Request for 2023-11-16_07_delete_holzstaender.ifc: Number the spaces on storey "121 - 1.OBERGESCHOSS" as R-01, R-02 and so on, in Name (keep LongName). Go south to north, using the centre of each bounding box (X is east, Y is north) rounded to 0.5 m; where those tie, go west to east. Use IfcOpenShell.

First a look at what the model holds.

```python
import ifcopenshell
import ifcopenshell.util.element
import ifcopenshell.util.placement

model = ifcopenshell.open("2023-11-16_07_delete_holzstaender.ifc")
print(model.schema)
storey = next(s for s in model.by_type("IfcBuildingStorey") if s.Name == "121 - 1.OBERGESCHOSS")
spaces = [e for e in ifcopenshell.util.element.get_decomposition(storey) if e.is_a("IfcSpace")]
for e in sorted(spaces, key=lambda e: e.id()):
    origin = ifcopenshell.util.placement.get_local_placement(e.ObjectPlacement)[:3, 3]
    print(e.id(), e.Name, e.LongName, origin.round(2) + 0.0, sep=" | ")
```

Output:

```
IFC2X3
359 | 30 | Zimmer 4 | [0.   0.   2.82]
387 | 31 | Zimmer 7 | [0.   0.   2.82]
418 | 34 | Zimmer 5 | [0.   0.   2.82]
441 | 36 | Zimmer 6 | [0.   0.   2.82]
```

```python
import ifcopenshell
import ifcopenshell.geom
import ifcopenshell.util.element
import ifcopenshell.util.shape

model = ifcopenshell.open("2023-11-16_07_delete_holzstaender.ifc")
settings = ifcopenshell.geom.settings()
settings.set("use-world-coords", True)


def centre(element):
    shape = ifcopenshell.geom.create_shape(settings, element)
    return ifcopenshell.util.shape.get_bbox_centroid(shape.geometry)


storey = next(s for s in model.by_type("IfcBuildingStorey") if s.Name == "121 - 1.OBERGESCHOSS")
spaces = [e for e in ifcopenshell.util.element.get_decomposition(storey) if e.is_a("IfcSpace")]

# Insertion points can sit at a corner or the storey origin, so sort by the geometry (in metres).
centres = {e: centre(e) for e in spaces}
spaces.sort(key=lambda e: (round(centres[e][1] / 0.5), centres[e][0]))

for i, e in enumerate(spaces, start=1):
    number = f"R-{i:02d}"
    e.Name = number
    print(e.id(), number)

model.write("2023-11-16_07_delete_holzstaender-out.ifc")
```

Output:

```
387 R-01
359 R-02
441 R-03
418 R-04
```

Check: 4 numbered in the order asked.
